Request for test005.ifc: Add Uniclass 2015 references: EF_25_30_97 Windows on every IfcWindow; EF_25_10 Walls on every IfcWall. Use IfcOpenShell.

First a look at what the model holds.

```python
import ifcopenshell

model = ifcopenshell.open("test005.ifc")
print(model.schema)
print("classifications:", [c.Name for c in model.by_type("IfcClassification")])
for ifc_class in ("IfcDoor", "IfcRoof", "IfcStair", "IfcWall", "IfcWindow"):
    print(ifc_class, len(model.by_type(ifc_class)))
```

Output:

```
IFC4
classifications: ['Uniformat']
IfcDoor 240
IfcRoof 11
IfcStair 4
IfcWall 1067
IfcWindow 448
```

```python
import ifcopenshell
import ifcopenshell.api.classification

model = ifcopenshell.open("test005.ifc")

system = ifcopenshell.api.classification.add_classification(model, classification="Uniclass 2015")

codes = {
    "IfcWindow": ("EF_25_30_97", "Windows"),
    "IfcWall": ("EF_25_10", "Walls"),
}
for ifc_class, (code, name) in codes.items():
    products = model.by_type(ifc_class)
    ifcopenshell.api.classification.add_reference(
        model, products=products, classification=system, identification=code, name=name
    )
    print(code, len(products))

model.write("test005_rev.ifc")
```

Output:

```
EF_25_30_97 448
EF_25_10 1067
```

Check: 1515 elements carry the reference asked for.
